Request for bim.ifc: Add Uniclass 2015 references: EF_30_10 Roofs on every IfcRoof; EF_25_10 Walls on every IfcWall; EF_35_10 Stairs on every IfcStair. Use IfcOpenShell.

First a look at what the model holds.

```python
import ifcopenshell

model = ifcopenshell.open("bim.ifc")
print(model.schema)
print("classifications:", [c.Name for c in model.by_type("IfcClassification")])
for ifc_class in ("IfcDoor", "IfcRoof", "IfcStair", "IfcWall", "IfcWindow"):
    print(ifc_class, len(model.by_type(ifc_class)))
```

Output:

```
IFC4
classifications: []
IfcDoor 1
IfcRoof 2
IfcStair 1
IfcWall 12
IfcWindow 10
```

```python
import ifcopenshell
import ifcopenshell.api.classification

model = ifcopenshell.open("bim.ifc")

system = ifcopenshell.api.classification.add_classification(model, classification="Uniclass 2015")

codes = {
    "IfcRoof": ("EF_30_10", "Roofs"),
    "IfcWall": ("EF_25_10", "Walls"),
    "IfcStair": ("EF_35_10", "Stairs"),
}
for ifc_class, (code, name) in codes.items():
    products = model.by_type(ifc_class)
    ifcopenshell.api.classification.add_reference(
        model, products=products, classification=system, identification=code, name=name
    )
    print(code, len(products))

model.write("bim_updated.ifc")
```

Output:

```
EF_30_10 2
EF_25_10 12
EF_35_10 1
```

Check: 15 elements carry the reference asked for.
